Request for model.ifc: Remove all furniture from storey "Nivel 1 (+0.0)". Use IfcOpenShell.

First a look at what the model holds.

```python
import ifcopenshell
import ifcopenshell.util.element

model = ifcopenshell.open("model.ifc")
print(model.schema)
storey = next(s for s in model.by_type("IfcBuildingStorey") if s.Name == "Nivel 1 (+0.0)")
furniture = [e for e in ifcopenshell.util.element.get_decomposition(storey) if e.is_a("IfcFurnishingElement")]
seen = {}
for e in furniture:
    element_type = ifcopenshell.util.element.get_type(e)
    name = element_type.Name if element_type not in (None, e) else None
    seen[name] = seen.get(name, 0) + 1
for name, count in sorted(seen.items(), key=str):
    print(count, "x", name)
```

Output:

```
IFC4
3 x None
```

```python
import ifcopenshell
import ifcopenshell.api.root
import ifcopenshell.util.element

model = ifcopenshell.open("model.ifc")

storey = next(s for s in model.by_type("IfcBuildingStorey") if s.Name == "Nivel 1 (+0.0)")
furniture = [e for e in ifcopenshell.util.element.get_decomposition(storey) if e.is_a("IfcFurnishingElement")]

for e in furniture:
    ifcopenshell.api.root.remove_product(model, product=e)
print(len(furniture), "removed")

model.write("model_rev.ifc")
```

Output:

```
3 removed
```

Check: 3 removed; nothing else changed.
